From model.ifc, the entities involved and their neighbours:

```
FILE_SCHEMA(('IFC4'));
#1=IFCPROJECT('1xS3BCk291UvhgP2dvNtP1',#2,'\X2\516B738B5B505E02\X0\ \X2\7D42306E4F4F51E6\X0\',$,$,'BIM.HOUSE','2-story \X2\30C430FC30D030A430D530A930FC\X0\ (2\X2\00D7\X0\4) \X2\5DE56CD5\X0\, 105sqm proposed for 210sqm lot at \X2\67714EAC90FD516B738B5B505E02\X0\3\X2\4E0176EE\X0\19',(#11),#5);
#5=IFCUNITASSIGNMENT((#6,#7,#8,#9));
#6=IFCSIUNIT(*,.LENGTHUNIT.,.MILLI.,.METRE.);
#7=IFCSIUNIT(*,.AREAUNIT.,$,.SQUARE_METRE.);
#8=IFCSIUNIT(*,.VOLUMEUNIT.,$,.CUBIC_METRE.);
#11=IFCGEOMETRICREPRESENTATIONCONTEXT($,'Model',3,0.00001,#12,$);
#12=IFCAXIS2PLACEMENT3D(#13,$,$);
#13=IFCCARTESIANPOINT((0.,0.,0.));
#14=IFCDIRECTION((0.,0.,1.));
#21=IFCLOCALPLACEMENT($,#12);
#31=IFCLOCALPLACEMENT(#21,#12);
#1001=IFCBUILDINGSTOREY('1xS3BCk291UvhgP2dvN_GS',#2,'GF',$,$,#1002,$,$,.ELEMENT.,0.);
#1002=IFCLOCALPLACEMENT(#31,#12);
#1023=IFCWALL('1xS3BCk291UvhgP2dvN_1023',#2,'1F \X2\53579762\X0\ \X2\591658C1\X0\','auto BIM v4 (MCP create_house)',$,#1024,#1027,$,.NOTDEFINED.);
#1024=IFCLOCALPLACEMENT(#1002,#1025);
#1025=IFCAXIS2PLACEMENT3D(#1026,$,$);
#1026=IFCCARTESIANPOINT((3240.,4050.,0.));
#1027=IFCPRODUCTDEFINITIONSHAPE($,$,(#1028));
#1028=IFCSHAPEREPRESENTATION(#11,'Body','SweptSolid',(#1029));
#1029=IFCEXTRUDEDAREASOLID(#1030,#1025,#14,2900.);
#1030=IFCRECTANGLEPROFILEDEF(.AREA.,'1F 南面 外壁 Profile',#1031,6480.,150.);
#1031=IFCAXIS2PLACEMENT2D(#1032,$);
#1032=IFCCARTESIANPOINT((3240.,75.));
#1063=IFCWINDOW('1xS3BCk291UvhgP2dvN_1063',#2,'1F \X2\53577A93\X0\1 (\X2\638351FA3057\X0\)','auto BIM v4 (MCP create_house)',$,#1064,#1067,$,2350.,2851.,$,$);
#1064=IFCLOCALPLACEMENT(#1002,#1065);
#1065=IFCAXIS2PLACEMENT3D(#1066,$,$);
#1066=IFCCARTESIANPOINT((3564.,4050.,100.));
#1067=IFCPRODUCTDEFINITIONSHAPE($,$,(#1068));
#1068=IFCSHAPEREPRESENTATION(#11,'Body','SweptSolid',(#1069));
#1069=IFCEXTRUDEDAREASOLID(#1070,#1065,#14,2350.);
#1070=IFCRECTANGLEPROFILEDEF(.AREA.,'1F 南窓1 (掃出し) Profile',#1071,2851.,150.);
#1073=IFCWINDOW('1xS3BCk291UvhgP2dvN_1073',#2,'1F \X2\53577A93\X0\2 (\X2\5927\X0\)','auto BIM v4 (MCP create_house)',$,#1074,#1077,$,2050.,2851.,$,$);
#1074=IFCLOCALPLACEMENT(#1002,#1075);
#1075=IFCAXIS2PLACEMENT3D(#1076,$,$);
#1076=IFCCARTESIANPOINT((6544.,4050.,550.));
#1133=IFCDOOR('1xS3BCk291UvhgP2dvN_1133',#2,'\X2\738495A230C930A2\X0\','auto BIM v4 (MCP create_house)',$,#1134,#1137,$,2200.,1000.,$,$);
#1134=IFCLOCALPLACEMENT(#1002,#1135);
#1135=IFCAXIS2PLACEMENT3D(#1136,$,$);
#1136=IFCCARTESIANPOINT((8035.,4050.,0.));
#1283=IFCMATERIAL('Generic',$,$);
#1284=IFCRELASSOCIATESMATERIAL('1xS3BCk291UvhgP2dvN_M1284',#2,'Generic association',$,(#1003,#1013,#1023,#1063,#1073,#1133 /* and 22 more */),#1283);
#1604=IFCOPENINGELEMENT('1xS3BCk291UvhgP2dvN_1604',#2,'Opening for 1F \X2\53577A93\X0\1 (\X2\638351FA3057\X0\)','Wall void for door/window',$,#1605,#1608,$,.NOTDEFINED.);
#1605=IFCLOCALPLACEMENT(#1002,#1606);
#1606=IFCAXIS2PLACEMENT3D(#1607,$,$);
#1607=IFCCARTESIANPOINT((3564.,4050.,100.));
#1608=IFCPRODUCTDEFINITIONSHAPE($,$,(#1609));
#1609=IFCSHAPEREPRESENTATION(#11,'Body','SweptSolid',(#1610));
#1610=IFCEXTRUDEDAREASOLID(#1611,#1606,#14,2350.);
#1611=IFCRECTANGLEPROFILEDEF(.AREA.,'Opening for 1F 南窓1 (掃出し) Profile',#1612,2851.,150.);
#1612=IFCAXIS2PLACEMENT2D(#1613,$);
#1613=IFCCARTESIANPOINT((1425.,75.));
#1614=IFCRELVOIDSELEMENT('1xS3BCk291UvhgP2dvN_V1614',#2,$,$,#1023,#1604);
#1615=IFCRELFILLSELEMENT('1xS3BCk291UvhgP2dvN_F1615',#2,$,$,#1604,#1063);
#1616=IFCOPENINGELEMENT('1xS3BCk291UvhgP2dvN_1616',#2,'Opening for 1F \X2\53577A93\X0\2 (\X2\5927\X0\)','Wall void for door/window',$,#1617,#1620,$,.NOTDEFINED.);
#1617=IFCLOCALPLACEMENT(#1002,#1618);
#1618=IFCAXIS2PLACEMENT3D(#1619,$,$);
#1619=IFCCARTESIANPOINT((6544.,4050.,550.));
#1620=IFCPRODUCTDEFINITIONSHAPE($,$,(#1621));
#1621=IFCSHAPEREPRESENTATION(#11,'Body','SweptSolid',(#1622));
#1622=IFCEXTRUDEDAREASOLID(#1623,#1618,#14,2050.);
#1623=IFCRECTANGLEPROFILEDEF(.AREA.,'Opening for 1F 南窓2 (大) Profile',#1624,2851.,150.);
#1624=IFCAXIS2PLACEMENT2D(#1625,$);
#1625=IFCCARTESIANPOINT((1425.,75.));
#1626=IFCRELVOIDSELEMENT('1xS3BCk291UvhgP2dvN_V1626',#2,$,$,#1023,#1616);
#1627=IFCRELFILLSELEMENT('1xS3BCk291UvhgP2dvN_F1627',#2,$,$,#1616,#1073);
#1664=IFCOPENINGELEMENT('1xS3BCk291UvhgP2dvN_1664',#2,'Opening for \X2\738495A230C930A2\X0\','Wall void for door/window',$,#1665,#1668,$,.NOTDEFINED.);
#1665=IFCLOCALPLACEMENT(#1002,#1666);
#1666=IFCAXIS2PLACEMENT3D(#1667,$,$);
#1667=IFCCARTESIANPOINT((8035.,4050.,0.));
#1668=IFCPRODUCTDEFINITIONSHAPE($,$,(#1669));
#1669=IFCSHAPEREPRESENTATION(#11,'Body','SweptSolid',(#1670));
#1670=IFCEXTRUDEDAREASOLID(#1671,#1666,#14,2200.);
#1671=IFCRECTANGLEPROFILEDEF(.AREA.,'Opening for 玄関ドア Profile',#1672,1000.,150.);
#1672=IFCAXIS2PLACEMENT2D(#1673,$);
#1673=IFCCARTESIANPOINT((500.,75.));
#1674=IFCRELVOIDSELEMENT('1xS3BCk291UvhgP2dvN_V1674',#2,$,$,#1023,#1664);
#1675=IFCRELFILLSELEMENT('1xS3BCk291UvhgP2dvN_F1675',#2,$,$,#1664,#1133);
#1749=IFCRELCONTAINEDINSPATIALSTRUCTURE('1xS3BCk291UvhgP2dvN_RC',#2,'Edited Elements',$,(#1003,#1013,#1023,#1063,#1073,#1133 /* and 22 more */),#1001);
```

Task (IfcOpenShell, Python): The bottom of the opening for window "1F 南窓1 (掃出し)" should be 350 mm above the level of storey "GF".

```python
import numpy as np
import ifcopenshell
import ifcopenshell.api.geometry
import ifcopenshell.geom
import ifcopenshell.util.element
import ifcopenshell.util.placement
import ifcopenshell.util.shape
import ifcopenshell.util.unit

model = ifcopenshell.open("model.ifc")
unit_scale = ifcopenshell.util.unit.calculate_unit_scale(model)

window = model.by_guid("1xS3BCk291UvhgP2dvN_1063")
opening = window.FillsVoids[0].RelatingOpeningElement
storey = ifcopenshell.util.element.get_container(window, ifc_class="IfcBuildingStorey")
level = ifcopenshell.util.placement.get_local_placement(storey.ObjectPlacement)[2, 3]

# The opening's origin need not be at the sill, so measure its lowest point.
shape = ifcopenshell.geom.create_shape(ifcopenshell.geom.settings(), opening)
bottom = ifcopenshell.util.shape.get_shape_bottom_elevation(shape, shape.geometry) / unit_scale
dz = level + 0.35 / unit_scale - bottom

shift = np.array([0.0, 0.0, dz])
# The window is not placed relative to its opening, so move both.
for product in (opening, window):
    matrix = ifcopenshell.util.placement.get_local_placement(product.ObjectPlacement)
    matrix[:3, 3] += shift
    ifcopenshell.api.geometry.edit_object_placement(model, product=product, matrix=matrix, is_si=False)

print(f"moved by {dz * unit_scale:+.3f} m")

model.write("model_rev.ifc")
```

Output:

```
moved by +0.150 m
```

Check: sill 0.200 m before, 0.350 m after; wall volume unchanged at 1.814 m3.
